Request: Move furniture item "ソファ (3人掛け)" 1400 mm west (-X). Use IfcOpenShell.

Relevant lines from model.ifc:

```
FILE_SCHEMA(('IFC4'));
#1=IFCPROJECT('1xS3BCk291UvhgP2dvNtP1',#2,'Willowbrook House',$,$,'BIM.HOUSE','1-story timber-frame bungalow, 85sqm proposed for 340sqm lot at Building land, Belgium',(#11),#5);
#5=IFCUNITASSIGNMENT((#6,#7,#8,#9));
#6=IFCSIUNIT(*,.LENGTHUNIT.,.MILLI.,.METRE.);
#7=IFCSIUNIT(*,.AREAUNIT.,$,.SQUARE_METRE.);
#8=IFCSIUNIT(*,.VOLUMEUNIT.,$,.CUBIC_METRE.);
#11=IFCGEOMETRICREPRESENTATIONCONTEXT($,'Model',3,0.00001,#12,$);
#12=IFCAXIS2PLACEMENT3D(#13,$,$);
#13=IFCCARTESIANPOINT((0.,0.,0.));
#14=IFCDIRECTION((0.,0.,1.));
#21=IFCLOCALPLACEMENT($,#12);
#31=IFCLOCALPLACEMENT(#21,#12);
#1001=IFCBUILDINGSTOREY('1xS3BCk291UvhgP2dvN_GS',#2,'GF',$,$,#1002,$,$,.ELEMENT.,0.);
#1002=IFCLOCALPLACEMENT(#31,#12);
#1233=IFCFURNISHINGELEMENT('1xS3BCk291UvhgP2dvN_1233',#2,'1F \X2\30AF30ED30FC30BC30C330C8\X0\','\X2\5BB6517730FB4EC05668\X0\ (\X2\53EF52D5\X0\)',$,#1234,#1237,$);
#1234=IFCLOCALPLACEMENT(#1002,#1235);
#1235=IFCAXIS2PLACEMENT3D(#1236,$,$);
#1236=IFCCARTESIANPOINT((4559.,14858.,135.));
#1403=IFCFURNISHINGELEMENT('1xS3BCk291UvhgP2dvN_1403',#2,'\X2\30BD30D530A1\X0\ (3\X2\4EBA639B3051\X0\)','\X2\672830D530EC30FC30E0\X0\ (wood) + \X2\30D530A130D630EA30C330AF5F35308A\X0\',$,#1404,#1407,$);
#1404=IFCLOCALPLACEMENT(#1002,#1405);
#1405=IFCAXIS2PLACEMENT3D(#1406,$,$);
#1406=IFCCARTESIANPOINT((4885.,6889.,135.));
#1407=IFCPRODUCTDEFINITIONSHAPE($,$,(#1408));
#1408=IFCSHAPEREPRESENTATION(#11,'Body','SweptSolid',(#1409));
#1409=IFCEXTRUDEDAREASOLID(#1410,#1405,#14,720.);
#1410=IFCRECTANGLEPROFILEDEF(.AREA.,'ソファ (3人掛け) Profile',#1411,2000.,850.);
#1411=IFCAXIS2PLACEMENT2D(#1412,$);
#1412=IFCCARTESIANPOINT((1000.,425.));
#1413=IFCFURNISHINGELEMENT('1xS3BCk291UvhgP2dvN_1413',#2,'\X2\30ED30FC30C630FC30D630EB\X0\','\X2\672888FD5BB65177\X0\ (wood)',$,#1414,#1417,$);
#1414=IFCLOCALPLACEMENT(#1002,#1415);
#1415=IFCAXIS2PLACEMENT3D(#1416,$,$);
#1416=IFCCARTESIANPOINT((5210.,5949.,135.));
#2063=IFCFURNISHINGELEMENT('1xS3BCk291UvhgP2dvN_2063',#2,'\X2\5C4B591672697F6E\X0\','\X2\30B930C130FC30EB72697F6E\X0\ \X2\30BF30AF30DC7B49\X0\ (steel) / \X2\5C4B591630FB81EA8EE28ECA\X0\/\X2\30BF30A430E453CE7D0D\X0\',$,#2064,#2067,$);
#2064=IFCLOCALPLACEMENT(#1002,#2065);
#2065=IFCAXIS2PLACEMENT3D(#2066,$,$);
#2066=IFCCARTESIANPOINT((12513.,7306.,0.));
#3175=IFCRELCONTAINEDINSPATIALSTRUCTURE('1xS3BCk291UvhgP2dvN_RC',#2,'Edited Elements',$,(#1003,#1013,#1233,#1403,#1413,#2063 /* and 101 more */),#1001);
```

```python
import ifcopenshell
import ifcopenshell.api.geometry
import ifcopenshell.util.placement

model = ifcopenshell.open("model.ifc")

item = model.by_guid("1xS3BCk291UvhgP2dvN_1403")
matrix = ifcopenshell.util.placement.get_local_placement(item.ObjectPlacement)
matrix[0, 3] -= 1400.0
ifcopenshell.api.geometry.edit_object_placement(model, product=item, matrix=matrix, is_si=False)

print(ifcopenshell.util.placement.get_local_placement(item.ObjectPlacement).round(3) + 0.0)

model.write("model_updated.ifc")
```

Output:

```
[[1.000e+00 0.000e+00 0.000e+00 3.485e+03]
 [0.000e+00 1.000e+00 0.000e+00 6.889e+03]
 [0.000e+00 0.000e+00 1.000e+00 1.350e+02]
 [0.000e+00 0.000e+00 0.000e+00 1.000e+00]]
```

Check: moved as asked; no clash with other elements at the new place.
